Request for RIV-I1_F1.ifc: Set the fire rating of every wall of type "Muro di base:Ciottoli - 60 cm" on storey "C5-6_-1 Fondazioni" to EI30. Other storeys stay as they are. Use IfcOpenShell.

First a look at what the model holds.

```python
import ifcopenshell
import ifcopenshell.util.element

model = ifcopenshell.open("RIV-I1_F1.ifc")
print(model.schema)
storey = next(s for s in model.by_type("IfcBuildingStorey") if s.Name == "C5-6_-1 Fondazioni")
walls = [e for e in ifcopenshell.util.element.get_decomposition(storey) if e.is_a("IfcWall")]
seen = {}
for e in walls:
    element_type = ifcopenshell.util.element.get_type(e)
    key = (element_type.Name if element_type != e and element_type else None, ifcopenshell.util.element.get_pset(e, "Pset_WallCommon", "FireRating"))
    seen[key] = seen.get(key, 0) + 1
for (name, value), count in sorted(seen.items(), key=str):
    print(count, "x", name, "|", value)
```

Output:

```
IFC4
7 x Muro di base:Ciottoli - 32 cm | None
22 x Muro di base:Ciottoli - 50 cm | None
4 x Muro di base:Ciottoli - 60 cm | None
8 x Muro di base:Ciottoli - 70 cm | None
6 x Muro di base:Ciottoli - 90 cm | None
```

```python
import ifcopenshell
import ifcopenshell.api.pset
import ifcopenshell.util.element

model = ifcopenshell.open("RIV-I1_F1.ifc")

storey = next(s for s in model.by_type("IfcBuildingStorey") if s.Name == "C5-6_-1 Fondazioni")
walls = [e for e in ifcopenshell.util.element.get_decomposition(storey) if e.is_a("IfcWall")]

count = 0
for e in walls:
    element_type = ifcopenshell.util.element.get_type(e)
    if element_type in (None, e) or element_type.Name != "Muro di base:Ciottoli - 60 cm":
        continue
    # add_pset returns the element's existing set when there is one.
    pset = ifcopenshell.api.pset.add_pset(model, product=e, name="Pset_WallCommon")
    ifcopenshell.api.pset.edit_pset(model, pset=pset, properties={"FireRating": "EI30"})
    count += 1

print(count, "walls updated")

model.write("RIV-I1_F1-out.ifc")
```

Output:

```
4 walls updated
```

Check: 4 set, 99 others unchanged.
